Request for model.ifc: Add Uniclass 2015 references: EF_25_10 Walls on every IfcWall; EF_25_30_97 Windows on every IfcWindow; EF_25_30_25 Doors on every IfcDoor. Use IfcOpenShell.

First a look at what the model holds.

```python
import ifcopenshell

model = ifcopenshell.open("model.ifc")
print(model.schema)
print("classifications:", [c.Name for c in model.by_type("IfcClassification")])
for ifc_class in ("IfcDoor", "IfcRoof", "IfcStair", "IfcWall", "IfcWindow"):
    print(ifc_class, len(model.by_type(ifc_class)))
```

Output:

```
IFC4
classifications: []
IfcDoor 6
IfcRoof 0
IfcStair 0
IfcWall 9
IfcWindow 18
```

```python
import ifcopenshell
import ifcopenshell.api.classification

model = ifcopenshell.open("model.ifc")

system = ifcopenshell.api.classification.add_classification(model, classification="Uniclass 2015")

codes = {
    "IfcWall": ("EF_25_10", "Walls"),
    "IfcWindow": ("EF_25_30_97", "Windows"),
    "IfcDoor": ("EF_25_30_25", "Doors"),
}
for ifc_class, (code, name) in codes.items():
    products = model.by_type(ifc_class)
    ifcopenshell.api.classification.add_reference(
        model, products=products, classification=system, identification=code, name=name
    )
    print(code, len(products))

model.write("model_v2.ifc")
```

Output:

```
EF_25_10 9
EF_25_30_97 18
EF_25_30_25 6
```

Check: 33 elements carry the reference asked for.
